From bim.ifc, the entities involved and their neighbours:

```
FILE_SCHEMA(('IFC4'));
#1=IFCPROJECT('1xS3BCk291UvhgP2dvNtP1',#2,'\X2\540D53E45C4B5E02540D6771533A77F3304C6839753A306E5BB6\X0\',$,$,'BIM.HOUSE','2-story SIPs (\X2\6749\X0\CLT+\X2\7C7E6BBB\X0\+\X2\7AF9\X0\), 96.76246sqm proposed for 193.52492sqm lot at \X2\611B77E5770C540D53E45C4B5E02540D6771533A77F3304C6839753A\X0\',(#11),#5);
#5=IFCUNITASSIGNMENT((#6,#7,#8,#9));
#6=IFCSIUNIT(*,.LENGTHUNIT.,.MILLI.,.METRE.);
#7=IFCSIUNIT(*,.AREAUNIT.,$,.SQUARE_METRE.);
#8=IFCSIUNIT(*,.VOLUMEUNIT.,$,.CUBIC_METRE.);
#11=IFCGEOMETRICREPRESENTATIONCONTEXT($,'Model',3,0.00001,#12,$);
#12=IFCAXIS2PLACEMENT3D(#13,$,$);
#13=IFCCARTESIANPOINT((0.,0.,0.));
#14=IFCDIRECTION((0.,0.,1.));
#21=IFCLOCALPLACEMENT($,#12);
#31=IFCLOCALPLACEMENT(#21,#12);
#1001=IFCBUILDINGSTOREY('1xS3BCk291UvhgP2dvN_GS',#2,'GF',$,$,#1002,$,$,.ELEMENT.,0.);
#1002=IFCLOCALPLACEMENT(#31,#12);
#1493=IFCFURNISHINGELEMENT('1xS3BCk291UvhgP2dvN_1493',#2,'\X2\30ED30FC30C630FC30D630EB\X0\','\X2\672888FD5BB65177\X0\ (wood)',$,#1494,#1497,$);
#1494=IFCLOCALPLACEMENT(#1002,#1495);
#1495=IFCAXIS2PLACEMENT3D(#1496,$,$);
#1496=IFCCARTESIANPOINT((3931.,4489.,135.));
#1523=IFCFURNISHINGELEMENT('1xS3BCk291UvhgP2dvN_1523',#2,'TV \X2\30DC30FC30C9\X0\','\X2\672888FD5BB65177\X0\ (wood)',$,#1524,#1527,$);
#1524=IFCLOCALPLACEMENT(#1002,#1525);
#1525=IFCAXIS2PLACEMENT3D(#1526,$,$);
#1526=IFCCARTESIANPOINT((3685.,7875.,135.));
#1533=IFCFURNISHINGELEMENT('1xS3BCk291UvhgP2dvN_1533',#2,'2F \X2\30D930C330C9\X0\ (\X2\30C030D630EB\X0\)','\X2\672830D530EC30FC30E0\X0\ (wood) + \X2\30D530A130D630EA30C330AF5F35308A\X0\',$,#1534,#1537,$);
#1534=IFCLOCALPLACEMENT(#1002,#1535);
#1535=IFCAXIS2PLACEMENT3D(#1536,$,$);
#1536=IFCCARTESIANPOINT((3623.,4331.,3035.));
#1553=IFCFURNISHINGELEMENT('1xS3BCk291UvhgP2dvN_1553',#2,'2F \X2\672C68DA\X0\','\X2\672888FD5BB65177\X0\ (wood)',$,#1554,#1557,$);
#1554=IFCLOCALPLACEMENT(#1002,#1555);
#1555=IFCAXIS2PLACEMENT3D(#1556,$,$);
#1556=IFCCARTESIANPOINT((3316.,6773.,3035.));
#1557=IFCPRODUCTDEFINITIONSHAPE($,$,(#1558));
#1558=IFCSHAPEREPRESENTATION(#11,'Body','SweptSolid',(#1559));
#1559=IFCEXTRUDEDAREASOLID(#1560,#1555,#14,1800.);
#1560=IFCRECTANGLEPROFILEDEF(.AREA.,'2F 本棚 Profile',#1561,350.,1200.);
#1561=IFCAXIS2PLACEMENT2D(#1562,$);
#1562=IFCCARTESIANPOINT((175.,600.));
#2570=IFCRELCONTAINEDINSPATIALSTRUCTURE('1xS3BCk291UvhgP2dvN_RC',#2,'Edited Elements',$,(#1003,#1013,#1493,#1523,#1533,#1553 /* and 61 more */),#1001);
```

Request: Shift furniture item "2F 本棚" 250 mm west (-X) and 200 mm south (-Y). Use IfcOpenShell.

```python
import ifcopenshell
import ifcopenshell.api.geometry
import ifcopenshell.util.placement

model = ifcopenshell.open("bim.ifc")

item = model.by_guid("1xS3BCk291UvhgP2dvN_1553")
matrix = ifcopenshell.util.placement.get_local_placement(item.ObjectPlacement)
matrix[0, 3] -= 250.0
matrix[1, 3] -= 200.0
ifcopenshell.api.geometry.edit_object_placement(model, product=item, matrix=matrix, is_si=False)

print(ifcopenshell.util.placement.get_local_placement(item.ObjectPlacement).round(3) + 0.0)

model.write("bim_rev.ifc")
```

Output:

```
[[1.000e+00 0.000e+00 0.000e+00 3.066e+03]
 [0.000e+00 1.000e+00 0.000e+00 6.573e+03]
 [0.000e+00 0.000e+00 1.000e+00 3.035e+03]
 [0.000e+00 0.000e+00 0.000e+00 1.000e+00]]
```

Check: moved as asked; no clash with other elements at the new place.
